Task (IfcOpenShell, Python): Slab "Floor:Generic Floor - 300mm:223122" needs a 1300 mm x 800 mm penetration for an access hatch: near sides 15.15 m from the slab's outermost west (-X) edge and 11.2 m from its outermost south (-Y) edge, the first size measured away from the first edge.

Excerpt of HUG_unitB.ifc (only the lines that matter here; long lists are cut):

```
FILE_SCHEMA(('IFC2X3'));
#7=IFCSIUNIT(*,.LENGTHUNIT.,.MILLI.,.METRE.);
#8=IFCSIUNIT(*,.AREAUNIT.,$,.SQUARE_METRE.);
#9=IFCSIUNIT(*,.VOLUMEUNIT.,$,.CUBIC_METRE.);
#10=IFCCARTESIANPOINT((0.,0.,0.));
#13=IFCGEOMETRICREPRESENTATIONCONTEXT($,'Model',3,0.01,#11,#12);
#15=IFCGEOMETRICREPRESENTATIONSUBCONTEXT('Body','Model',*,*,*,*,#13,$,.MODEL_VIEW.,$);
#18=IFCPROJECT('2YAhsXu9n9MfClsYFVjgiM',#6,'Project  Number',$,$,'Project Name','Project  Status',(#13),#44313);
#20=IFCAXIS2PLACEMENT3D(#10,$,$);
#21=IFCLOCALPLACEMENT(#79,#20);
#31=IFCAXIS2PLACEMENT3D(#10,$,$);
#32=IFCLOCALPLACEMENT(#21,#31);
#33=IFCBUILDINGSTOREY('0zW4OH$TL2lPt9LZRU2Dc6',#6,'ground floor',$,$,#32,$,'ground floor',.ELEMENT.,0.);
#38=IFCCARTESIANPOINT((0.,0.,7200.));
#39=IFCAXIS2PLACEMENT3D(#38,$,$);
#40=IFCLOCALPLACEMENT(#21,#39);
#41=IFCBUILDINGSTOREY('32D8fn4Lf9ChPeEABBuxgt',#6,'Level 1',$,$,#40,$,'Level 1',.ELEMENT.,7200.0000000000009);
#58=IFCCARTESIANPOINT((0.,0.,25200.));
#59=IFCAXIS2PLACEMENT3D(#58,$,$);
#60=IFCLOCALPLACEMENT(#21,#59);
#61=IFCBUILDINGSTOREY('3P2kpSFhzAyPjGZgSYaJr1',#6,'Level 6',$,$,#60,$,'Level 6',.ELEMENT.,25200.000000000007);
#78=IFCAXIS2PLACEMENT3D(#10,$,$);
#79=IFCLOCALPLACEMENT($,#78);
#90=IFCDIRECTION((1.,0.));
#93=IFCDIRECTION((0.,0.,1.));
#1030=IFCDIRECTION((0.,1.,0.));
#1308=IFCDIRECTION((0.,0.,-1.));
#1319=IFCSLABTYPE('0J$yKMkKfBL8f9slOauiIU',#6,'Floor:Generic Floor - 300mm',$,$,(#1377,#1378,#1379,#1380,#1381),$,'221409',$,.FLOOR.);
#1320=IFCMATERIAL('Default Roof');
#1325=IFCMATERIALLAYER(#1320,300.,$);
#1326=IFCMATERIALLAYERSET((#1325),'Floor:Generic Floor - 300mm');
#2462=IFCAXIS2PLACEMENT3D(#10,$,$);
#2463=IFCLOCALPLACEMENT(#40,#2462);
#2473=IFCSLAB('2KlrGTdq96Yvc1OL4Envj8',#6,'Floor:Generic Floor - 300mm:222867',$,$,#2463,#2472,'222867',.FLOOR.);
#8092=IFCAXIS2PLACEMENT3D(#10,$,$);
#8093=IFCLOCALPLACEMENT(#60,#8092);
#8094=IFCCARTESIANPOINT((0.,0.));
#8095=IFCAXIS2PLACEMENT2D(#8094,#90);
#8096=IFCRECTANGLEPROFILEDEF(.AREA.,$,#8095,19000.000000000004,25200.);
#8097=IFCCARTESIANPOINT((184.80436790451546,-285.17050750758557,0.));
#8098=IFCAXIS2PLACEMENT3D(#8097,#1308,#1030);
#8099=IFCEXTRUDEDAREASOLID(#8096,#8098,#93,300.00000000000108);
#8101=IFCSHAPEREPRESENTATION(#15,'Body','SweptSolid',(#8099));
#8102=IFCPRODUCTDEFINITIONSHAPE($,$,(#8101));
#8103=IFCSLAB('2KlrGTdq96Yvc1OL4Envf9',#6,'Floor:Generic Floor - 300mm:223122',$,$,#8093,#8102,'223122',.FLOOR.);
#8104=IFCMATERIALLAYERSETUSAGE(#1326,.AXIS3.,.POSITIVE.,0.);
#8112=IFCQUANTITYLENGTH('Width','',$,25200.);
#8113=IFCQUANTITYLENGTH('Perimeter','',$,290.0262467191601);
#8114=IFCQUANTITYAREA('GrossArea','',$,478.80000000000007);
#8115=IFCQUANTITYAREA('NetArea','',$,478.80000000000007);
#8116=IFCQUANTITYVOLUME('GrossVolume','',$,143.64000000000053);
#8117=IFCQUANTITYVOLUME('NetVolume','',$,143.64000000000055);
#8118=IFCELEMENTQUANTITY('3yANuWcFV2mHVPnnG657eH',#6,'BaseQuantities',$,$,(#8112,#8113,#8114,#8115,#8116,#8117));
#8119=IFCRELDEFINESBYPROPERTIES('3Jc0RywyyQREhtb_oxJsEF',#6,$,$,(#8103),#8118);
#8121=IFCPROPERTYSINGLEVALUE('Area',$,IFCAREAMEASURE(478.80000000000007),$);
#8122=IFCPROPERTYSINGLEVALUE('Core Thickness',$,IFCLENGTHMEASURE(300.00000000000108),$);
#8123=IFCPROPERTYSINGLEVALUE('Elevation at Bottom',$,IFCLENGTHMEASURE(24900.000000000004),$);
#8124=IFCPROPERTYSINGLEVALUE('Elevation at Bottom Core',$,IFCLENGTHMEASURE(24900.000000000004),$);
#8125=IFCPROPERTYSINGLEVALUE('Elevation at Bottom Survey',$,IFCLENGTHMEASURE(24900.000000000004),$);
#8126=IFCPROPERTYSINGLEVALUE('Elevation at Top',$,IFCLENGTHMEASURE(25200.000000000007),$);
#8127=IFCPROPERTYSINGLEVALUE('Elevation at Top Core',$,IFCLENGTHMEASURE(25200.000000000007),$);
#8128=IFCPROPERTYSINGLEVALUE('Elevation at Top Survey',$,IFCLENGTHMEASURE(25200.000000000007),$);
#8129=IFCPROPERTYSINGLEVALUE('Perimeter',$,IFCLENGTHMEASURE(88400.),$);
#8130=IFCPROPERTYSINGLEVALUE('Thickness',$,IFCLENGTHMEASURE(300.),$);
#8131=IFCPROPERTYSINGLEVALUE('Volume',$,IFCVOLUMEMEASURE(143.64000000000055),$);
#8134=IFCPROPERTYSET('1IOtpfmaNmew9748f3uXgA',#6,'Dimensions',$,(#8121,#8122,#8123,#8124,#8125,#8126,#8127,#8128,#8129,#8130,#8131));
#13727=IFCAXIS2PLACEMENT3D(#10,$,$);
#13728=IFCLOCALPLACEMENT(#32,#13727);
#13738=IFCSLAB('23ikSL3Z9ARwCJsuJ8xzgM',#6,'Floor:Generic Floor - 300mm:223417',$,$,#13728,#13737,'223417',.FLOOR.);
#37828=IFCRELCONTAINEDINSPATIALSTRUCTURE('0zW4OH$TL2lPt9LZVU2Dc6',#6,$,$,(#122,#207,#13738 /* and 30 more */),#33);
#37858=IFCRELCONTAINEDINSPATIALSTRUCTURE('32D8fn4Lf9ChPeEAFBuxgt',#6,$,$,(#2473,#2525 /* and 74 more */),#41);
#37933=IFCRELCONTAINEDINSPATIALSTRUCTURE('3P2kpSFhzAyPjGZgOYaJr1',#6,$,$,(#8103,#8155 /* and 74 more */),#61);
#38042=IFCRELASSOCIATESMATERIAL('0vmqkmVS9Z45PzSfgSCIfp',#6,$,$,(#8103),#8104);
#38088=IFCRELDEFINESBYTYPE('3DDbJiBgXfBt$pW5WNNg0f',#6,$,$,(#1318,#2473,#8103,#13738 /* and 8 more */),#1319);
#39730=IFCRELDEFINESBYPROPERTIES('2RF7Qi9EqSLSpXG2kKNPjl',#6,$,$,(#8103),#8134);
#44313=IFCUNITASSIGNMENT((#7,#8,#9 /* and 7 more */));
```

```python
import numpy as np
import ifcopenshell
import ifcopenshell.api.feature
import ifcopenshell.api.geometry
import ifcopenshell.api.pset
import ifcopenshell.api.root
import ifcopenshell.geom
import ifcopenshell.util.element
import ifcopenshell.util.placement
import ifcopenshell.util.representation
import ifcopenshell.util.shape
import ifcopenshell.util.unit

model = ifcopenshell.open("HUG_unitB.ifc")
unit_scale = ifcopenshell.util.unit.calculate_unit_scale(model)
area_scale = ifcopenshell.util.unit.calculate_unit_scale(model, "AREAUNIT")
volume_scale = ifcopenshell.util.unit.calculate_unit_scale(model, "VOLUMEUNIT")
settings = ifcopenshell.geom.settings()


def volume(element):
    """Net volume in cubic metres, openings subtracted."""
    shape = ifcopenshell.geom.create_shape(settings, element)
    return ifcopenshell.util.shape.get_volume(shape.geometry)


slab = model.by_id(8103)
before = volume(slab)

# Extent in the slab's own axes, in metres. The edges named are its -X and -Y sides.
slab_shape = ifcopenshell.geom.create_shape(settings, slab)
vertices = ifcopenshell.util.shape.get_vertices(slab_shape.geometry)
x_min, y_min, bottom = vertices.min(axis=0)
top = vertices[:, 2].max()

opening = ifcopenshell.api.root.create_entity(model, ifc_class="IfcOpeningElement", name="Access hatch opening")
context = ifcopenshell.util.representation.get_context(model, "Model", "Body", "MODEL_VIEW")
width, depth = 1.3, 0.8
outline = [(0.0, 0.0), (width, 0.0), (width, depth), (0.0, depth), (0.0, 0.0)]
# Overshoot both faces by 50 mm so the cut is clean.
shape = ifcopenshell.api.geometry.add_slab_representation(
    model, context=context, depth=top - bottom + 0.1, polyline=outline
)
ifcopenshell.api.geometry.assign_representation(model, product=opening, representation=shape)

matrix = ifcopenshell.util.placement.get_local_placement(slab.ObjectPlacement)
matrix[:, 3] = matrix @ np.append(np.array([x_min + 15.15, y_min + 11.2, bottom - 0.05]) / unit_scale, 1.0)
ifcopenshell.api.geometry.edit_object_placement(model, product=opening, matrix=matrix, is_si=False)
ifcopenshell.api.feature.add_feature(model, feature=opening, element=slab)

after = volume(slab)

# Update the slab's stored quantities.
qto = model.by_id(ifcopenshell.util.element.get_pset(slab, "BaseQuantities", should_inherit=False)["id"])
ifcopenshell.api.pset.edit_qto(model, qto=qto, properties={
    "NetArea": after / (top - bottom) / area_scale,
    "NetVolume": after / volume_scale,
})
pset = model.by_id(ifcopenshell.util.element.get_pset(slab, "Dimensions", should_inherit=False)["id"])
ifcopenshell.api.pset.edit_pset(model, pset=pset, properties={
    "Area": model.create_entity("IfcAreaMeasure", after / (top - bottom) / area_scale),
    "Volume": model.create_entity("IfcVolumeMeasure", after / volume_scale),
})

print(f"slab volume {before:.3f} -> {after:.3f} m3")

model.write("HUG_unitB_v2.ifc")
```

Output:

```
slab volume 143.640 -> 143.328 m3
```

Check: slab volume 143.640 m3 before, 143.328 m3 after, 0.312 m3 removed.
